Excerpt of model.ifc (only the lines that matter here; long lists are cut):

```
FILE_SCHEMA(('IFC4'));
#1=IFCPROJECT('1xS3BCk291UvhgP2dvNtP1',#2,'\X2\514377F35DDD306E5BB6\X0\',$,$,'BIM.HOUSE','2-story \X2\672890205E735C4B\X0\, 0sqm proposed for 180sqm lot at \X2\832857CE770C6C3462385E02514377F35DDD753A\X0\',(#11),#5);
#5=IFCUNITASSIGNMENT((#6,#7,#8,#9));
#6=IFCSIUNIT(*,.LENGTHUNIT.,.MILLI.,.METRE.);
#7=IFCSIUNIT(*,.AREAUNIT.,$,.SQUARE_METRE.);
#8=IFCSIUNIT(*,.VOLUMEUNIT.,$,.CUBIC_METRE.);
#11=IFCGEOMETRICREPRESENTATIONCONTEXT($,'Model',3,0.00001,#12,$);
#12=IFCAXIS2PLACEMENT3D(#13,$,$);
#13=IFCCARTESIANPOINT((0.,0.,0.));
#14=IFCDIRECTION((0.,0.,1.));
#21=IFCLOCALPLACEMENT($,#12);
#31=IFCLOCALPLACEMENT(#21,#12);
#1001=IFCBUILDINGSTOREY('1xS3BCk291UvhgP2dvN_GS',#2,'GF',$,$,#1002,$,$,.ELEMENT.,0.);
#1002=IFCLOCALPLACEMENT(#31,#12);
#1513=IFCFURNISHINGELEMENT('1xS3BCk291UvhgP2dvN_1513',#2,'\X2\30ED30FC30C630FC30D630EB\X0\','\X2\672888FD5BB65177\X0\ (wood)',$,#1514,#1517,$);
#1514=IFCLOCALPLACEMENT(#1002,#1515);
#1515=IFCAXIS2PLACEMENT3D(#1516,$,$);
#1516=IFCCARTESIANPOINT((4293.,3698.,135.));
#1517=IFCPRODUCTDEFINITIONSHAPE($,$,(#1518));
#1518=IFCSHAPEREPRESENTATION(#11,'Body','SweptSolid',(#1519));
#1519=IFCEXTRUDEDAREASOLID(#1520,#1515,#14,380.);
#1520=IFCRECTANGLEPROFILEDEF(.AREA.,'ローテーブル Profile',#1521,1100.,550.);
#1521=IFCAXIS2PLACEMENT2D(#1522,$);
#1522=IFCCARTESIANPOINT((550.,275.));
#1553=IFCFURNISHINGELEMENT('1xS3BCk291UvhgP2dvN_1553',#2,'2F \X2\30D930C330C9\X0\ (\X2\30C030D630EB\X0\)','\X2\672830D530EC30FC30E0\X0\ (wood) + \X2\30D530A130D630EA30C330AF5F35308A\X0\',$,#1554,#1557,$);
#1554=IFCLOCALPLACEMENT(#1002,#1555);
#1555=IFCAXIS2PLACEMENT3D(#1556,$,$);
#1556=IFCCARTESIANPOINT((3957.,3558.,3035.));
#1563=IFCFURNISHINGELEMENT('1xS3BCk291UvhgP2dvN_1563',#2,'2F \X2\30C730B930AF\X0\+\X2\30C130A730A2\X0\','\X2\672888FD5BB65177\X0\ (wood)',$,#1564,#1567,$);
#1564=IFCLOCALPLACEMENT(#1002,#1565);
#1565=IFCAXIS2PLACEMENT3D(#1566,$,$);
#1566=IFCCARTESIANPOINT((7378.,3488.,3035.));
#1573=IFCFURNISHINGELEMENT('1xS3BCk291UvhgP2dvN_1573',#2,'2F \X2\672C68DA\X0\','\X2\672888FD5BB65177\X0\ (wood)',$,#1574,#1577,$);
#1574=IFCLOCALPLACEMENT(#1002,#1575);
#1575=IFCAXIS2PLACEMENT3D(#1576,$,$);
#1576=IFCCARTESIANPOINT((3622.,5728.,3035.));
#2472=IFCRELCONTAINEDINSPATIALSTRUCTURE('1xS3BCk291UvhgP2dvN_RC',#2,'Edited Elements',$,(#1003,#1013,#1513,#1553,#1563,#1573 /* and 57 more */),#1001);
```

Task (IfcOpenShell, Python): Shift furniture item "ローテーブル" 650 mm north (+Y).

```python
import ifcopenshell
import ifcopenshell.api.geometry
import ifcopenshell.util.placement
import ifcopenshell.util.unit

model = ifcopenshell.open("model.ifc")
unit_scale = ifcopenshell.util.unit.calculate_unit_scale(model)

item = model.by_guid("1xS3BCk291UvhgP2dvN_1513")
matrix = ifcopenshell.util.placement.get_local_placement(item.ObjectPlacement)
matrix[1, 3] += 0.65 / unit_scale
ifcopenshell.api.geometry.edit_object_placement(model, product=item, matrix=matrix, is_si=False)

print(ifcopenshell.util.placement.get_local_placement(item.ObjectPlacement).round(3) + 0.0)

model.write("model_v2.ifc")
```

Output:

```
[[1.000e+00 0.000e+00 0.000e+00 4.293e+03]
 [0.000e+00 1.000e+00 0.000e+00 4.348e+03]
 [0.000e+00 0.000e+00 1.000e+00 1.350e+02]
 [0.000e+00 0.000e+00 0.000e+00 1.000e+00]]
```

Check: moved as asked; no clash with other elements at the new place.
